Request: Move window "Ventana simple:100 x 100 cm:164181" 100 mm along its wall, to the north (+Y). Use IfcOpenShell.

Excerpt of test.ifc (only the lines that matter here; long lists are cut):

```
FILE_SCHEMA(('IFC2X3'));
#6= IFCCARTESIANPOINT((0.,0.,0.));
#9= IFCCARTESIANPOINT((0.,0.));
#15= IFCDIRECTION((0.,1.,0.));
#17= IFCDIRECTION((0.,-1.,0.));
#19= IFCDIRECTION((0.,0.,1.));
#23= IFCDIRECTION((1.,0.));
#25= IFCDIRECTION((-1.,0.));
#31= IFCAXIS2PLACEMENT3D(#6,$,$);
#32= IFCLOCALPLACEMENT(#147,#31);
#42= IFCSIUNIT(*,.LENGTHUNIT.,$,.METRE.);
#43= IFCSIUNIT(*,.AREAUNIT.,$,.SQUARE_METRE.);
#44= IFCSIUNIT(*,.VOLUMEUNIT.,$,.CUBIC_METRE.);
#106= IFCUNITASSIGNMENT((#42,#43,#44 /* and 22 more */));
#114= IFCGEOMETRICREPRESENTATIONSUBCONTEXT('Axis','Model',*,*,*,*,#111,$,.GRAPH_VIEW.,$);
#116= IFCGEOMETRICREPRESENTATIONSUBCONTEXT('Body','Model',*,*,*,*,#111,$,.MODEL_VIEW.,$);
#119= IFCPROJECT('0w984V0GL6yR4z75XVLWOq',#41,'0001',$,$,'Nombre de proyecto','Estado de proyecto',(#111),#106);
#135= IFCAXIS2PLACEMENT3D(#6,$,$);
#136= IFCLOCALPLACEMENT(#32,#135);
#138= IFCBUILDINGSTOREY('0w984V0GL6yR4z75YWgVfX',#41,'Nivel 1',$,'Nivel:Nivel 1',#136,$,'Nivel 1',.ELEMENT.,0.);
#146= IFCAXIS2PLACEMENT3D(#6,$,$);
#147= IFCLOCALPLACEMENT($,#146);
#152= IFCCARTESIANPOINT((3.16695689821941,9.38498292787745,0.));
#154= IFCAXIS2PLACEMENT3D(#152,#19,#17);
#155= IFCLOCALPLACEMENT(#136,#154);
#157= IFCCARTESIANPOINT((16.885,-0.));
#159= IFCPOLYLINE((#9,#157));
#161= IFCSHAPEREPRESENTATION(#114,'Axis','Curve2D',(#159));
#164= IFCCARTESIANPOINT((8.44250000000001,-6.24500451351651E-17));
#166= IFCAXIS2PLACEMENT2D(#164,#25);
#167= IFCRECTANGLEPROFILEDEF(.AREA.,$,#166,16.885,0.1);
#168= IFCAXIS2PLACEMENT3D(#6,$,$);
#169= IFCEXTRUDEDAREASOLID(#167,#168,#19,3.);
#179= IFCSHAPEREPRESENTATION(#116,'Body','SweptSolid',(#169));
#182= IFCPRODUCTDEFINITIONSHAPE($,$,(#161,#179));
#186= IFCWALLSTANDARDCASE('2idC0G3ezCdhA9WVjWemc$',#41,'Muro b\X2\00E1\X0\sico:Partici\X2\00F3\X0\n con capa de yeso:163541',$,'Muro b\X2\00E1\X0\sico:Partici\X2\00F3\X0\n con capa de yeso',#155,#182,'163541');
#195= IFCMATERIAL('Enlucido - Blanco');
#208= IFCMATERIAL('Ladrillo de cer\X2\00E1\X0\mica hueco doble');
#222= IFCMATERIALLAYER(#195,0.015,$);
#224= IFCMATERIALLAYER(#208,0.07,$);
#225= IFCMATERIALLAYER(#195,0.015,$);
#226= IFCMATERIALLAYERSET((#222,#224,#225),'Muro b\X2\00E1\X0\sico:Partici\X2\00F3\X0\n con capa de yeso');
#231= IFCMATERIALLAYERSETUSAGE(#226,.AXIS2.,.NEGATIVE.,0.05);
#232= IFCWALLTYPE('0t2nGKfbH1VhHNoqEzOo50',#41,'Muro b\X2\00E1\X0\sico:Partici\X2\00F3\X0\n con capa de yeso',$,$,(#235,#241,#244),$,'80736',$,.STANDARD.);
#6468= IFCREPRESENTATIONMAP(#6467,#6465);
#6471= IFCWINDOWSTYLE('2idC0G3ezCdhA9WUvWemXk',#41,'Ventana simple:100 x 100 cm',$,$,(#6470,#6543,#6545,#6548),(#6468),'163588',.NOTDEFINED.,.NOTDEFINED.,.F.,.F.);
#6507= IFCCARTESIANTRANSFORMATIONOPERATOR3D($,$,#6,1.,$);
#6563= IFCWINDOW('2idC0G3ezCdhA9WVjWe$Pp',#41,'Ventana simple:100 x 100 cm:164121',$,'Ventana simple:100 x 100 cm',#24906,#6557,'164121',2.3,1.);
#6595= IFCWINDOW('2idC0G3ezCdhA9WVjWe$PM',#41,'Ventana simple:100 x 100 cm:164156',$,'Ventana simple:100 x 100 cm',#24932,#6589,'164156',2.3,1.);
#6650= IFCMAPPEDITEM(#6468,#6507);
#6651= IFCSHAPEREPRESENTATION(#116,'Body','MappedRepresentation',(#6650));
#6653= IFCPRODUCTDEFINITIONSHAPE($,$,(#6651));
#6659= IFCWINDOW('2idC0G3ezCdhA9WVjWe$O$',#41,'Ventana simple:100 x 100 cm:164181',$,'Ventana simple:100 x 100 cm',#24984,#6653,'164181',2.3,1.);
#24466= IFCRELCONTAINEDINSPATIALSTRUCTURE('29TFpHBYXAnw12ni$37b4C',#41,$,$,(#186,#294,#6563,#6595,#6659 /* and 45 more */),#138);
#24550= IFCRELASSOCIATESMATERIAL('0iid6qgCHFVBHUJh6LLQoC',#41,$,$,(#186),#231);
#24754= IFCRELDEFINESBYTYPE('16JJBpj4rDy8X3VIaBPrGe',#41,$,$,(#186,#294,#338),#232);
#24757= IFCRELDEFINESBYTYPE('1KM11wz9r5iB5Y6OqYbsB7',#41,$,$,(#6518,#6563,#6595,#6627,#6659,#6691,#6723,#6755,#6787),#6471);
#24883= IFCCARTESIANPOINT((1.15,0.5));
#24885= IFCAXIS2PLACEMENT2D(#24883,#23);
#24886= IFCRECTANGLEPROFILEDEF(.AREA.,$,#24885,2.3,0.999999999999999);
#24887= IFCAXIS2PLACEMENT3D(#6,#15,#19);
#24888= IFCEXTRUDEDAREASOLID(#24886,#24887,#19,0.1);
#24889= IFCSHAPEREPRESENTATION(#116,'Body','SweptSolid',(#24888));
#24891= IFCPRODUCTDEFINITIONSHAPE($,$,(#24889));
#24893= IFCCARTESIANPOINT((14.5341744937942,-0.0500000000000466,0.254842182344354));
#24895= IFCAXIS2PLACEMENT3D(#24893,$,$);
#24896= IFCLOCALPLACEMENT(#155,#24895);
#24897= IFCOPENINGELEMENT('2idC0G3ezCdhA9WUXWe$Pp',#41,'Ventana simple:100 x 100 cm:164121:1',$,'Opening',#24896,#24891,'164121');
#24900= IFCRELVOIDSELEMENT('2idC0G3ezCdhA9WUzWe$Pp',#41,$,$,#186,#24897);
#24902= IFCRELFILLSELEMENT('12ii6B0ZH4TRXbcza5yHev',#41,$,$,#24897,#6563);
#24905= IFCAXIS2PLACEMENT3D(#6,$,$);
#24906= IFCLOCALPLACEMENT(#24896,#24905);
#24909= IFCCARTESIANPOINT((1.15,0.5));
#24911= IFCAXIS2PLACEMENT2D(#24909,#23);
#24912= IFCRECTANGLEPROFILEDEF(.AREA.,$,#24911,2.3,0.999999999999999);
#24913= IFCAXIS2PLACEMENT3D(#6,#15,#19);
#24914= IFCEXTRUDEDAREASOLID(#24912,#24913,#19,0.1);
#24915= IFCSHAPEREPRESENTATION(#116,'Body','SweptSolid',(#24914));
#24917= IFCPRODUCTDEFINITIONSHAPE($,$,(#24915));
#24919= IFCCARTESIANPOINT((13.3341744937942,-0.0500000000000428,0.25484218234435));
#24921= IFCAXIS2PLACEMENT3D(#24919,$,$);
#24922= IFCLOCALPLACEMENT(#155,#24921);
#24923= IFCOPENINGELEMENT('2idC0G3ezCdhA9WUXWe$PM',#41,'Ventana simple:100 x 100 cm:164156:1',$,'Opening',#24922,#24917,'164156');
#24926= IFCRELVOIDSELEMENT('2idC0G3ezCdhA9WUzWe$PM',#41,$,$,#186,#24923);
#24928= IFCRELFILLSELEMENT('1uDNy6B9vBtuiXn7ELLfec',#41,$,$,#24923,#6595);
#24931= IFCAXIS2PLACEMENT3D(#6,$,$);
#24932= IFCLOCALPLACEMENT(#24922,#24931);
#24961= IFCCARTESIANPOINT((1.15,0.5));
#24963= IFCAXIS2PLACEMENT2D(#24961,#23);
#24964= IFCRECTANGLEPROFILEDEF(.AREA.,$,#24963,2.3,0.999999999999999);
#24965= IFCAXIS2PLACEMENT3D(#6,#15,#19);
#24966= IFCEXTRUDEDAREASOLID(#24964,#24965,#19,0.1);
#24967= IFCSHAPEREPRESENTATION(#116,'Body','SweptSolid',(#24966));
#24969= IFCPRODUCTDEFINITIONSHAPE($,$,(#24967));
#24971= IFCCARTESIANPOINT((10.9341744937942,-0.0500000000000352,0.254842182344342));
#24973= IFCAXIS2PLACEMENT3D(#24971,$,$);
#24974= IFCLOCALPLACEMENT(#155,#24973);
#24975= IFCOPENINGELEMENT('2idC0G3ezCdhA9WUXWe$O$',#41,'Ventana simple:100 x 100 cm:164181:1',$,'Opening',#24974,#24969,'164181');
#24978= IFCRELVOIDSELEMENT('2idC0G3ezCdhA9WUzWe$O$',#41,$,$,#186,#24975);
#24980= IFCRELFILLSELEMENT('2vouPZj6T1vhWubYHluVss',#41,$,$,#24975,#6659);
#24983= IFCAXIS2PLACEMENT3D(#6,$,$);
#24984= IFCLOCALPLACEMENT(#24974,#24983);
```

```python
import ifcopenshell
import ifcopenshell.api.geometry
import ifcopenshell.util.placement
import ifcopenshell.util.unit

model = ifcopenshell.open("test.ifc")
unit_scale = ifcopenshell.util.unit.calculate_unit_scale(model)

window = model.by_guid("2idC0G3ezCdhA9WVjWe$O$")
opening = window.FillsVoids[0].RelatingOpeningElement
wall = opening.VoidsElements[0].RelatingBuildingElement

wall_matrix = ifcopenshell.util.placement.get_local_placement(wall.ObjectPlacement)
shift = wall_matrix[:3, 0] * -0.1 / unit_scale
before = ifcopenshell.util.placement.get_local_placement(window.ObjectPlacement)[:3, 3].copy()

# The window is placed relative to its opening, so it follows when the opening moves.
matrix = ifcopenshell.util.placement.get_local_placement(opening.ObjectPlacement)
matrix[:3, 3] += shift
ifcopenshell.api.geometry.edit_object_placement(
    model, product=opening, matrix=matrix, is_si=False, should_transform_children=True
)

after = ifcopenshell.util.placement.get_local_placement(window.ObjectPlacement)[:3, 3]
print("window moved by", (after - before).round(3) + 0.0)

model.write("test_v2.ifc")
```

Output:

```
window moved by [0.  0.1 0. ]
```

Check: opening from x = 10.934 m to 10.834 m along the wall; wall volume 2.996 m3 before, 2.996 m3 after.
